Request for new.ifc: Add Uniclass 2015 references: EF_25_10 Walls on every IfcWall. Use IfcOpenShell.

First a look at what the model holds.

```python
import ifcopenshell

model = ifcopenshell.open("new.ifc")
print(model.schema)
print("classifications:", [c.Name for c in model.by_type("IfcClassification")])
for ifc_class in ("IfcDoor", "IfcRoof", "IfcStair", "IfcWall", "IfcWindow"):
    print(ifc_class, len(model.by_type(ifc_class)))
```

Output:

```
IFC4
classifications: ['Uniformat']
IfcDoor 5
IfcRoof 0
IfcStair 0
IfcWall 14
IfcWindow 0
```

```python
import ifcopenshell
import ifcopenshell.api.classification

model = ifcopenshell.open("new.ifc")

system = ifcopenshell.api.classification.add_classification(model, classification="Uniclass 2015")

codes = {
    "IfcWall": ("EF_25_10", "Walls"),
}
for ifc_class, (code, name) in codes.items():
    products = model.by_type(ifc_class)
    ifcopenshell.api.classification.add_reference(
        model, products=products, classification=system, identification=code, name=name
    )
    print(code, len(products))

model.write("new_v2.ifc")
```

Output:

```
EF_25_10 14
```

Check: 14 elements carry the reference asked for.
